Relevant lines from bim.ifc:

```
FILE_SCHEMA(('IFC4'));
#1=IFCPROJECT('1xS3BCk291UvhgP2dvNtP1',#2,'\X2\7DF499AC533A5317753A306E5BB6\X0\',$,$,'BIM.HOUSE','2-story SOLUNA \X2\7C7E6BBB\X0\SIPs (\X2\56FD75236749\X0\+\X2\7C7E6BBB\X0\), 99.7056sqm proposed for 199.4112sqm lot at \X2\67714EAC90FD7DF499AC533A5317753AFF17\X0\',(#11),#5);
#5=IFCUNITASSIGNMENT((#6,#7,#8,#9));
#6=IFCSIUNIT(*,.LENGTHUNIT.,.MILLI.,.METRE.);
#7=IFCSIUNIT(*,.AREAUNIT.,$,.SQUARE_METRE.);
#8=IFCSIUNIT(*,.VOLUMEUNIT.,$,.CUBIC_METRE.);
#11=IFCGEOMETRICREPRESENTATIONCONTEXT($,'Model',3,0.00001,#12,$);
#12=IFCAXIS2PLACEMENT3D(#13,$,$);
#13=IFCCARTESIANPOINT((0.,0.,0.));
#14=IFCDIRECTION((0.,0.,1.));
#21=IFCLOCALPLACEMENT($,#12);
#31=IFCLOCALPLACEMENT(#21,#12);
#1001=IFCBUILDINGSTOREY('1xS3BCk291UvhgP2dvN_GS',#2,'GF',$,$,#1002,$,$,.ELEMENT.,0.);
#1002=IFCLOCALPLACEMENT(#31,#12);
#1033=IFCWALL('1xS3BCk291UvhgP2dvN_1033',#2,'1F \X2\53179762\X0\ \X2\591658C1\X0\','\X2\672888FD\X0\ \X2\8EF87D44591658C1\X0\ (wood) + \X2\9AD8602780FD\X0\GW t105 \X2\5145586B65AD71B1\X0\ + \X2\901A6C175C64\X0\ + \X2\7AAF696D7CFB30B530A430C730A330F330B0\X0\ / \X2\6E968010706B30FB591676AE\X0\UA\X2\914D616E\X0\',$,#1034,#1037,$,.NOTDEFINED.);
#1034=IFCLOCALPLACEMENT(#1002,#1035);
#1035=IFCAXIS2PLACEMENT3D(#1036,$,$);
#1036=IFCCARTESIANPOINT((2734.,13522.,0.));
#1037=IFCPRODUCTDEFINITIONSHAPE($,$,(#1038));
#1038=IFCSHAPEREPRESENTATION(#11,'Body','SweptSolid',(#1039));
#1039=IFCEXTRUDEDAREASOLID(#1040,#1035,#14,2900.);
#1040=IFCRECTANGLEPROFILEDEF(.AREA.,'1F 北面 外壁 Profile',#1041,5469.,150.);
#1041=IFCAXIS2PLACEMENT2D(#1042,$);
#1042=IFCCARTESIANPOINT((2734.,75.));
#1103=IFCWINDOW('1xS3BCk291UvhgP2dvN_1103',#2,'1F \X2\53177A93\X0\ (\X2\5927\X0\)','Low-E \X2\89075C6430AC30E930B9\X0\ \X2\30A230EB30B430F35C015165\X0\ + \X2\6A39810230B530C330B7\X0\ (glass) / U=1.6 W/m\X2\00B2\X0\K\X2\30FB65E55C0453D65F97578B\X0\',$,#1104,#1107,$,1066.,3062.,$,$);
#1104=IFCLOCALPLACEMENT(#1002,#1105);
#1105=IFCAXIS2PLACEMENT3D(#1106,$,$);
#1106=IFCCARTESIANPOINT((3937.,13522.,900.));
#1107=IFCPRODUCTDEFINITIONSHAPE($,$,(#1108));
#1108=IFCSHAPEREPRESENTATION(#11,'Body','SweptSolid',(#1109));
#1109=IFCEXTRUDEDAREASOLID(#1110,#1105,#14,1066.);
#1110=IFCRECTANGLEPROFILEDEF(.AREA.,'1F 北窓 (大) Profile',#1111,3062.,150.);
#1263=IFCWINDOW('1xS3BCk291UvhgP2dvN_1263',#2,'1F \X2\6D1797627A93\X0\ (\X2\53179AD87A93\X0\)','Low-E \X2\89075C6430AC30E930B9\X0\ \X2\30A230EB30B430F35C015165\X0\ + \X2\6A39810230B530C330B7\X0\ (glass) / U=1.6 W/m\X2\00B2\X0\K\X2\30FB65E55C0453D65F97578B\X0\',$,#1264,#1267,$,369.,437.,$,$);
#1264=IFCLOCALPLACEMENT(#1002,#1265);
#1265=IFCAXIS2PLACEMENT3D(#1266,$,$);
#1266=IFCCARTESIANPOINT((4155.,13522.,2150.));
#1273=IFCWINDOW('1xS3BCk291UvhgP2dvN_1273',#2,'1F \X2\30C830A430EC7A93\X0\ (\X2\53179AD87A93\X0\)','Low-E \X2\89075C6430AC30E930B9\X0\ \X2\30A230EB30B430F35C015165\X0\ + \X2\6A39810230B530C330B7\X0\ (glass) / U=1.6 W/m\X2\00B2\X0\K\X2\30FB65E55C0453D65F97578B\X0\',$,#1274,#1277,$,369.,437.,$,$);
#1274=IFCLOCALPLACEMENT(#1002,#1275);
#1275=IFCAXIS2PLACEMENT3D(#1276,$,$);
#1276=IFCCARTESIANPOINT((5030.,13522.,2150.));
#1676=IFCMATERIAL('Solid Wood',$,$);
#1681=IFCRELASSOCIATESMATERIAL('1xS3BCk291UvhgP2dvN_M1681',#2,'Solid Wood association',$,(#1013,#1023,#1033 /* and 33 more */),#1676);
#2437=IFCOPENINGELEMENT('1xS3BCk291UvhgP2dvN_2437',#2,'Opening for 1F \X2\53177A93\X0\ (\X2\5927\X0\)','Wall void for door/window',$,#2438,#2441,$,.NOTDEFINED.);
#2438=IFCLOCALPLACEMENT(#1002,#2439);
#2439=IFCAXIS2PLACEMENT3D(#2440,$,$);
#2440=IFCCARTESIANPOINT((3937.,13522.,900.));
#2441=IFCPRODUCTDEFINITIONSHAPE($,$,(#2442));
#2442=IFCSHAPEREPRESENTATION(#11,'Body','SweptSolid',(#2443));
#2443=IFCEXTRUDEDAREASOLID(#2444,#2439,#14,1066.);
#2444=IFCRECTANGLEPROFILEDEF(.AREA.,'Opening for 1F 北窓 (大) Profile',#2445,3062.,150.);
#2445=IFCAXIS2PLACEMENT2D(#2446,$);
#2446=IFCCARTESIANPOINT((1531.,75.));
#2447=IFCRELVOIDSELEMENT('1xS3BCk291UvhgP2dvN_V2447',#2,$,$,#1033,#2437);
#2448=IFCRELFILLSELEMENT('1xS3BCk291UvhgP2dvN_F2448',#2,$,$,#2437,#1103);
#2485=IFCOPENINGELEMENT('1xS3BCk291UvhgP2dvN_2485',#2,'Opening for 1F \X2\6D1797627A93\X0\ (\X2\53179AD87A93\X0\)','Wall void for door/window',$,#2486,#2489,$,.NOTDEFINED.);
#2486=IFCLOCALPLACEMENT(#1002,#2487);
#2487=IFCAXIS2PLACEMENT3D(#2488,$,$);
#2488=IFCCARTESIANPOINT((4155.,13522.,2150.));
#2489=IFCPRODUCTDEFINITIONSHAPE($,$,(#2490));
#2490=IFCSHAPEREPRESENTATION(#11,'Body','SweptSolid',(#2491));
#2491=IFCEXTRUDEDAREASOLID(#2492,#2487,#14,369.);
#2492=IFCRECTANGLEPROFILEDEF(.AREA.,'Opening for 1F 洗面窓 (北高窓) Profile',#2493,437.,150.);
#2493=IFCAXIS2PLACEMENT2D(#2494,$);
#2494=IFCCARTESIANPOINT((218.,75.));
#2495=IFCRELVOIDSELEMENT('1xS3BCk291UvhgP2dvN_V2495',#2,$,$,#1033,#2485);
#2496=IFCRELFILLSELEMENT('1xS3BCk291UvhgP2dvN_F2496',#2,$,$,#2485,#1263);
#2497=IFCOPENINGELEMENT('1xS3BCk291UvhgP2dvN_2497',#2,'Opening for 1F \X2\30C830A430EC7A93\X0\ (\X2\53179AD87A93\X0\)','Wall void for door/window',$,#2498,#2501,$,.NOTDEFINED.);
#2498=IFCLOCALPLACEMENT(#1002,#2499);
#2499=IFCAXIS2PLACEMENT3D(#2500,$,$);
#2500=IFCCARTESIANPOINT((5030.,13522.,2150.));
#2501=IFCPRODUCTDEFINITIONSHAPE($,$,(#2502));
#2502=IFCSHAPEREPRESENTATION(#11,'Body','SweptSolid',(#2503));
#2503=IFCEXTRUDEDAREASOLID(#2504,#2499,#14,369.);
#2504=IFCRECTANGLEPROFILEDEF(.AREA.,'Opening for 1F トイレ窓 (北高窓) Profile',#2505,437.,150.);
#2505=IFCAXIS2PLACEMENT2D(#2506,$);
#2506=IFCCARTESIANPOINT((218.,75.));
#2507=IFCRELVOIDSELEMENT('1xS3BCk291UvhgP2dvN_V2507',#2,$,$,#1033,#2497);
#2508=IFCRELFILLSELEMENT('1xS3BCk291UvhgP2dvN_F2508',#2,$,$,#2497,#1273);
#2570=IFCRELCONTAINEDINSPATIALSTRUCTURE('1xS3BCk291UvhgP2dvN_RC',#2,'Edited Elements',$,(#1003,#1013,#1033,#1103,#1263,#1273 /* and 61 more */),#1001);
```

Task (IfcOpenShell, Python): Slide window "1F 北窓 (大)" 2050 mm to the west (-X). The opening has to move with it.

```python
import ifcopenshell
import ifcopenshell.api.geometry
import ifcopenshell.util.placement
import ifcopenshell.util.unit

model = ifcopenshell.open("bim.ifc")
unit_scale = ifcopenshell.util.unit.calculate_unit_scale(model)

window = model.by_id(1103)
opening = window.FillsVoids[0].RelatingOpeningElement
wall = opening.VoidsElements[0].RelatingBuildingElement

wall_matrix = ifcopenshell.util.placement.get_local_placement(wall.ObjectPlacement)
shift = wall_matrix[:3, 0] * -2.05 / unit_scale
before = ifcopenshell.util.placement.get_local_placement(window.ObjectPlacement)[:3, 3].copy()

# The window is not placed relative to its opening, so move both.
for product in (opening, window):
    matrix = ifcopenshell.util.placement.get_local_placement(product.ObjectPlacement)
    matrix[:3, 3] += shift
    ifcopenshell.api.geometry.edit_object_placement(model, product=product, matrix=matrix, is_si=False)

after = ifcopenshell.util.placement.get_local_placement(window.ObjectPlacement)[:3, 3]
print("window moved by", (after - before).round(3) + 0.0)

model.write("bim_updated.ifc")
```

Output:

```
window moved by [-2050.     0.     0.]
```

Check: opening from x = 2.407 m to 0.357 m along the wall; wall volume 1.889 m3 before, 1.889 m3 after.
